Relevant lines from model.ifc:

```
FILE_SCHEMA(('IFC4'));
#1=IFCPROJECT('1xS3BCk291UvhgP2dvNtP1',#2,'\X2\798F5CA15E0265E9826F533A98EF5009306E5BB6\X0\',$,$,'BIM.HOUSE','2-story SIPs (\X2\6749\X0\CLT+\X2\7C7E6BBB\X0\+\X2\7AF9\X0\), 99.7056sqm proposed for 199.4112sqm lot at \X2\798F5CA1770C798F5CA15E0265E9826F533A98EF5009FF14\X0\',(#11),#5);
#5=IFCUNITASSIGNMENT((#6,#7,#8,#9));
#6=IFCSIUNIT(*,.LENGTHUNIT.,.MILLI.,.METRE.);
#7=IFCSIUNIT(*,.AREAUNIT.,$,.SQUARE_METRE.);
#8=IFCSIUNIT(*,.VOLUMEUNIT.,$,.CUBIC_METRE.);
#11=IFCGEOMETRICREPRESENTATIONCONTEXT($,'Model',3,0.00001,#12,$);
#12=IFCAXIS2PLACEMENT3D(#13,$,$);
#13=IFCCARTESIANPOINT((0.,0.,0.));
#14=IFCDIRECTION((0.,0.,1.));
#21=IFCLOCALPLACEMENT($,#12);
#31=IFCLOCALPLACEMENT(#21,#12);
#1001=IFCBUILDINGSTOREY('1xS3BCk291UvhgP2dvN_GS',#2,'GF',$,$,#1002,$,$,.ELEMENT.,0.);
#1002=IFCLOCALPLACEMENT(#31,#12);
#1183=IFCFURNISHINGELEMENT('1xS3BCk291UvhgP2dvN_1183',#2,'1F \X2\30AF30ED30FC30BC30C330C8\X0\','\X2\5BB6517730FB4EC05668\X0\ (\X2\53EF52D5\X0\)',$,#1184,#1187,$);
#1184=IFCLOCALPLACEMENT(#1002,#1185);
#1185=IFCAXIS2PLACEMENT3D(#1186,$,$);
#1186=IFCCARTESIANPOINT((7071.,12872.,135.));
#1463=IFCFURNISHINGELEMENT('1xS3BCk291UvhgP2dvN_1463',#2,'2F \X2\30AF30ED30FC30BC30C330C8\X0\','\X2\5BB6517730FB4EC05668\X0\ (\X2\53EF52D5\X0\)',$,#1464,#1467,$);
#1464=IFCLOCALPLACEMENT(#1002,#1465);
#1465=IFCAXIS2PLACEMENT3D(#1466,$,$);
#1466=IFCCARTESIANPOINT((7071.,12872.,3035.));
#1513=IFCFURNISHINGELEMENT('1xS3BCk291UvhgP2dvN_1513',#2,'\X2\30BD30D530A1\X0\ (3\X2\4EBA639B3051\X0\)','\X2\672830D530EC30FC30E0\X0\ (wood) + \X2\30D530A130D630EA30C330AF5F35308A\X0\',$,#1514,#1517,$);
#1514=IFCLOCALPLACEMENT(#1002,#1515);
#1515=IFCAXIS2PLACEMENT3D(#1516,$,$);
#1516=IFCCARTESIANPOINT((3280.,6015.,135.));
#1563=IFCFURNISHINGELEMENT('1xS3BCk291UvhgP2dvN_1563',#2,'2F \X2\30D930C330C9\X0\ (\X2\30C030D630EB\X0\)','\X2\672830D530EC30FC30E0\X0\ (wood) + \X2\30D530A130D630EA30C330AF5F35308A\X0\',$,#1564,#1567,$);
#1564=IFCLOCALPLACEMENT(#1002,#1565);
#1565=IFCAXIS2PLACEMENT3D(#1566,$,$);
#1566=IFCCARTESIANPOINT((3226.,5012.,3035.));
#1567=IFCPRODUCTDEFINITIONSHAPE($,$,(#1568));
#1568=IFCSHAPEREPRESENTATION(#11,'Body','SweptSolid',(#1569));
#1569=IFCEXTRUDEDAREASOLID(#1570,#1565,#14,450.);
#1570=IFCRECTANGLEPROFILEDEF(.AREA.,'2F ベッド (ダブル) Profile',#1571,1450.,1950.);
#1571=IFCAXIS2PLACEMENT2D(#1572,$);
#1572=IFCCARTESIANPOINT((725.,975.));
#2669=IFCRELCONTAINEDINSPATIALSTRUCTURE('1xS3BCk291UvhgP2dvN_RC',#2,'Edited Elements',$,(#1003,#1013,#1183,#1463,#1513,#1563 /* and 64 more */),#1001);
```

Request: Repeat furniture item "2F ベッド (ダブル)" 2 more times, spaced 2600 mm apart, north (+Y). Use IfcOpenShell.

```python
import numpy as np
import ifcopenshell
import ifcopenshell.api.geometry
import ifcopenshell.api.root
import ifcopenshell.util.element
import ifcopenshell.util.placement
import ifcopenshell.util.unit

model = ifcopenshell.open("model.ifc")
unit_scale = ifcopenshell.util.unit.calculate_unit_scale(model)


def reuse_history(source, copy):
    """copy_class also copies each property set's owner history, people and application; keep the originals."""
    for rel in copy.IsDefinedBy:
        if rel.is_a("IfcRelDefinesByProperties") and (history := rel.RelatingPropertyDefinition.OwnerHistory):
            rel.RelatingPropertyDefinition.OwnerHistory = source.OwnerHistory
            ifcopenshell.util.element.remove_deep2(model, history)


source = model.by_guid("1xS3BCk291UvhgP2dvN_1563")
base = ifcopenshell.util.placement.get_local_placement(source.ObjectPlacement)
step = np.array([0.0, 1.0, 0.0]) * 2.6 / unit_scale

for i in range(1, 3):
    copy = ifcopenshell.api.root.copy_class(model, product=source)
    copy.Representation = ifcopenshell.util.element.copy_deep(
        model, source.Representation, exclude=["IfcGeometricRepresentationContext", "IfcRepresentationMap"]
    )
    reuse_history(source, copy)
    matrix = base.copy()
    matrix[:3, 3] += i * step
    print("added at", matrix[:3, 3].round(3) + 0.0)
    ifcopenshell.api.geometry.edit_object_placement(model, product=copy, matrix=matrix, is_si=False)

model.write("model_updated.ifc")
```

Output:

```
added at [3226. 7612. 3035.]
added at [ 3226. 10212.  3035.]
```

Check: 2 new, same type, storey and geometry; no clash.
